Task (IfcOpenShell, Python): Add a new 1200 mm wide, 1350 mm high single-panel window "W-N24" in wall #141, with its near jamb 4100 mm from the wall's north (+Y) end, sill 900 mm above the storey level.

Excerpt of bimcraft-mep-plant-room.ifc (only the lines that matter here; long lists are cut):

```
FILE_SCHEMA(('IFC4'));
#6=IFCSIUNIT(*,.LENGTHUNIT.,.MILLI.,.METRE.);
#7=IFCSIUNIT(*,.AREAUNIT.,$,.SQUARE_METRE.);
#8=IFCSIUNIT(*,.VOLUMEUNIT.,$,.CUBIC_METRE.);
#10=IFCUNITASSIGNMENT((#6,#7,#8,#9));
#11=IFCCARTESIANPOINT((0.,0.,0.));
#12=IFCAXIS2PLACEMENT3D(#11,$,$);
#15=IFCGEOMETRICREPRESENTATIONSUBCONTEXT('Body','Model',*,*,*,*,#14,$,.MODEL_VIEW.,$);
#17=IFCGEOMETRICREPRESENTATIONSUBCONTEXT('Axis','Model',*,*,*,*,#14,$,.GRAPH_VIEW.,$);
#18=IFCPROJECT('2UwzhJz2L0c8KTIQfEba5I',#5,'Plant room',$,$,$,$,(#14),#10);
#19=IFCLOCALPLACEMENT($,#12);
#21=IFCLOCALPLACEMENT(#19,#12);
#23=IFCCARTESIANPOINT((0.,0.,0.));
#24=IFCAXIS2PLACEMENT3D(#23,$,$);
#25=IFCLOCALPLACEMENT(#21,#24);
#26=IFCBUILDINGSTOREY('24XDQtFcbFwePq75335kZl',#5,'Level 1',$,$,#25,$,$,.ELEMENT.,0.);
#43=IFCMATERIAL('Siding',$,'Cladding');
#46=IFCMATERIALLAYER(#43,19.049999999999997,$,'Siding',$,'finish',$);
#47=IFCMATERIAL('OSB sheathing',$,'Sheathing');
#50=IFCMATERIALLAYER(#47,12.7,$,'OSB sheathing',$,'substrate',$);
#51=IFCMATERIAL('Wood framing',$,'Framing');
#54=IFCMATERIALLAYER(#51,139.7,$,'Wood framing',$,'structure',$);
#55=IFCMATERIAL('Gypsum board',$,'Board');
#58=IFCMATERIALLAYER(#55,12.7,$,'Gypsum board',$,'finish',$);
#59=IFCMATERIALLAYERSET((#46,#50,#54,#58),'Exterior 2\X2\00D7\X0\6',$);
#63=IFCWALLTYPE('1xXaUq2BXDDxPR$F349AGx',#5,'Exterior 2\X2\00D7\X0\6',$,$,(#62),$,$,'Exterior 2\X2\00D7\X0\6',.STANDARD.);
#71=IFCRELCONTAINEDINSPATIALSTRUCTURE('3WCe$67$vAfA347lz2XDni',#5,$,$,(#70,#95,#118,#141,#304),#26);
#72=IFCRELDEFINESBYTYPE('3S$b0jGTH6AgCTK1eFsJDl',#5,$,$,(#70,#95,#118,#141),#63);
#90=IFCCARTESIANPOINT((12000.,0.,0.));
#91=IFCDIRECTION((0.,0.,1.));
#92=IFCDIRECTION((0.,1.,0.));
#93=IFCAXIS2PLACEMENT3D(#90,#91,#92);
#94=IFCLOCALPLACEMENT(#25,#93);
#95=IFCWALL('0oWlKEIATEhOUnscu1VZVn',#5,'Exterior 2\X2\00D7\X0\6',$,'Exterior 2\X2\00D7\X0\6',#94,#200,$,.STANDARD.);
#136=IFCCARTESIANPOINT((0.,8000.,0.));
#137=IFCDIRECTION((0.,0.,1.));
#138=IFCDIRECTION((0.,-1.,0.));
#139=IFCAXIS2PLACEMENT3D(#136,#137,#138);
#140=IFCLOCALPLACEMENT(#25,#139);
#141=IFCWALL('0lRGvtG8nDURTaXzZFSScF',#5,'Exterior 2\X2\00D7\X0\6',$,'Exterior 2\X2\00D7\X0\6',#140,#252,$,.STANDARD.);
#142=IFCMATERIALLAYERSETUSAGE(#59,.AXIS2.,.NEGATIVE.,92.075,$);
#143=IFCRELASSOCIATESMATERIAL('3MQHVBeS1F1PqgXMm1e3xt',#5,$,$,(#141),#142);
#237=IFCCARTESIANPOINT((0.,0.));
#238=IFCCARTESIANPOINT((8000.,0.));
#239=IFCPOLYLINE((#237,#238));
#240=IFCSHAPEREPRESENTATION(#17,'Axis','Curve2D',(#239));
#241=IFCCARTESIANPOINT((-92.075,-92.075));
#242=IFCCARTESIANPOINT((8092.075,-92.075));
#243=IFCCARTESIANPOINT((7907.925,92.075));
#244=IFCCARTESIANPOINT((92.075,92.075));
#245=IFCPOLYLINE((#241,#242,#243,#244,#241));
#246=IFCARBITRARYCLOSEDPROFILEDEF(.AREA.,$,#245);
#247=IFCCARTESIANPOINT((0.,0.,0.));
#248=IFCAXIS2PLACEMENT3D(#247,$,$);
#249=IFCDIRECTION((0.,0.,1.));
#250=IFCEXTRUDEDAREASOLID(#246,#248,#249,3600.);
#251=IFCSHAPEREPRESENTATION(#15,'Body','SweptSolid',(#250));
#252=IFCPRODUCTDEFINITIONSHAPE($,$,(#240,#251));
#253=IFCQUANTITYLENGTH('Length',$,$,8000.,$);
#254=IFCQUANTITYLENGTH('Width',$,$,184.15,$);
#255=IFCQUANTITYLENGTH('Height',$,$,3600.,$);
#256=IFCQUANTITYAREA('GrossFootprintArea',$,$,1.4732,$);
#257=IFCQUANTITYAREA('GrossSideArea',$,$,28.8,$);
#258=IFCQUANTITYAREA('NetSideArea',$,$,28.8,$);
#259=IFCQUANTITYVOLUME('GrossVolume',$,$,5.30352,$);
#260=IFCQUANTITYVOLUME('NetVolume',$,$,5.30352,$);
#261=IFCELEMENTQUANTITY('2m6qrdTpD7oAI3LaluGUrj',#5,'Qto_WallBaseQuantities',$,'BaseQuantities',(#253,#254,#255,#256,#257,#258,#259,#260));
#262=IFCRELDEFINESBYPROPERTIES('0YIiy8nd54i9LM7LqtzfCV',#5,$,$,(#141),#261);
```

```python
import numpy as np
import ifcopenshell
import ifcopenshell.api.feature
import ifcopenshell.api.geometry
import ifcopenshell.api.pset
import ifcopenshell.api.root
import ifcopenshell.api.spatial
import ifcopenshell.geom
import ifcopenshell.util.element
import ifcopenshell.util.placement
import ifcopenshell.util.representation
import ifcopenshell.util.shape
import ifcopenshell.util.unit

model = ifcopenshell.open("bimcraft-mep-plant-room.ifc")
unit_scale = ifcopenshell.util.unit.calculate_unit_scale(model)
area_scale = ifcopenshell.util.unit.calculate_unit_scale(model, "AREAUNIT")
volume_scale = ifcopenshell.util.unit.calculate_unit_scale(model, "VOLUMEUNIT")
settings = ifcopenshell.geom.settings()


def volume(element):
    """Net volume in cubic metres, openings subtracted."""
    shape = ifcopenshell.geom.create_shape(settings, element)
    return ifcopenshell.util.shape.get_volume(shape.geometry)


wall = model.by_id(141)
storey = ifcopenshell.util.element.get_container(wall, ifc_class="IfcBuildingStorey")
context = ifcopenshell.util.representation.get_context(model, "Model", "Body", "MODEL_VIEW")
before = volume(wall)

width, height, from_end, sill = 1.2, 1.35, 4.1, 0.9  # metres

# The wall runs along its own X axis, and the end named is its -X end.
wall_shape = ifcopenshell.geom.create_shape(settings, wall)
x, y, z = ifcopenshell.util.shape.get_vertices(wall_shape.geometry).T
start = x.min() + from_end
face, thickness = float(y.min()), float(y.max() - y.min())
wall_matrix = ifcopenshell.util.placement.get_local_placement(wall.ObjectPlacement)
level = ifcopenshell.util.placement.get_local_placement(storey.ObjectPlacement)[2, 3]


def in_wall(x, y):
    """Placement at x, y metres in the wall's axes, at sill height."""
    matrix = wall_matrix.copy()
    matrix[:, 3] = wall_matrix @ np.array([x / unit_scale, y / unit_scale, 0.0, 1.0])
    matrix[2, 3] = level + sill / unit_scale
    return matrix


# Opening: a box that overshoots both wall faces by 50 mm.
opening = ifcopenshell.api.root.create_entity(model, ifc_class="IfcOpeningElement", predefined_type="OPENING")
box = ifcopenshell.api.geometry.add_wall_representation(
    model, context=context, length=width, height=height, thickness=thickness + 0.1
)
ifcopenshell.api.geometry.assign_representation(model, product=opening, representation=box)
ifcopenshell.api.geometry.edit_object_placement(model, product=opening, matrix=in_wall(start, face - 0.05), is_si=False)
ifcopenshell.api.feature.add_feature(model, feature=opening, element=wall)

window = ifcopenshell.api.root.create_entity(model, ifc_class="IfcWindow", name="W-N24", predefined_type="WINDOW")
window.OverallWidth, window.OverallHeight = width / unit_scale, height / unit_scale
window.PartitioningType = "SINGLE_PANEL"
body = ifcopenshell.api.geometry.add_window_representation(
    model,
    context=context,
    overall_width=window.OverallWidth,
    overall_height=window.OverallHeight,
    partition_type="SINGLE_PANEL",
)
ifcopenshell.api.geometry.assign_representation(model, product=window, representation=body)
ifcopenshell.api.spatial.assign_container(model, products=[window], relating_structure=storey)
ifcopenshell.api.feature.add_filling(model, opening=opening, element=window)

# Centre the window in the wall's thickness.
ifcopenshell.api.geometry.edit_object_placement(model, product=window, matrix=in_wall(start, face), is_si=False)
window_shape = ifcopenshell.geom.create_shape(settings, window)
depth = ifcopenshell.util.shape.get_vertices(window_shape.geometry)[:, 1]
offset = face + thickness / 2 - (depth.min() + depth.max()) / 2
ifcopenshell.api.geometry.edit_object_placement(model, product=window, matrix=in_wall(start, offset), is_si=False)

after = volume(wall)

# Update the wall's stored quantities.
qto = model.by_id(ifcopenshell.util.element.get_pset(wall, "Qto_WallBaseQuantities", should_inherit=False)["id"])
ifcopenshell.api.pset.edit_qto(model, qto=qto, properties={
    "NetSideArea": after / thickness / area_scale,
    "NetVolume": after / volume_scale,
})

print(f"wall volume {before:.3f} -> {after:.3f} m3")

model.write("bimcraft-mep-plant-room_edited.ifc")
```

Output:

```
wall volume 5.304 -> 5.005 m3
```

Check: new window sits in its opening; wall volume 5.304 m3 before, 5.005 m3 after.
